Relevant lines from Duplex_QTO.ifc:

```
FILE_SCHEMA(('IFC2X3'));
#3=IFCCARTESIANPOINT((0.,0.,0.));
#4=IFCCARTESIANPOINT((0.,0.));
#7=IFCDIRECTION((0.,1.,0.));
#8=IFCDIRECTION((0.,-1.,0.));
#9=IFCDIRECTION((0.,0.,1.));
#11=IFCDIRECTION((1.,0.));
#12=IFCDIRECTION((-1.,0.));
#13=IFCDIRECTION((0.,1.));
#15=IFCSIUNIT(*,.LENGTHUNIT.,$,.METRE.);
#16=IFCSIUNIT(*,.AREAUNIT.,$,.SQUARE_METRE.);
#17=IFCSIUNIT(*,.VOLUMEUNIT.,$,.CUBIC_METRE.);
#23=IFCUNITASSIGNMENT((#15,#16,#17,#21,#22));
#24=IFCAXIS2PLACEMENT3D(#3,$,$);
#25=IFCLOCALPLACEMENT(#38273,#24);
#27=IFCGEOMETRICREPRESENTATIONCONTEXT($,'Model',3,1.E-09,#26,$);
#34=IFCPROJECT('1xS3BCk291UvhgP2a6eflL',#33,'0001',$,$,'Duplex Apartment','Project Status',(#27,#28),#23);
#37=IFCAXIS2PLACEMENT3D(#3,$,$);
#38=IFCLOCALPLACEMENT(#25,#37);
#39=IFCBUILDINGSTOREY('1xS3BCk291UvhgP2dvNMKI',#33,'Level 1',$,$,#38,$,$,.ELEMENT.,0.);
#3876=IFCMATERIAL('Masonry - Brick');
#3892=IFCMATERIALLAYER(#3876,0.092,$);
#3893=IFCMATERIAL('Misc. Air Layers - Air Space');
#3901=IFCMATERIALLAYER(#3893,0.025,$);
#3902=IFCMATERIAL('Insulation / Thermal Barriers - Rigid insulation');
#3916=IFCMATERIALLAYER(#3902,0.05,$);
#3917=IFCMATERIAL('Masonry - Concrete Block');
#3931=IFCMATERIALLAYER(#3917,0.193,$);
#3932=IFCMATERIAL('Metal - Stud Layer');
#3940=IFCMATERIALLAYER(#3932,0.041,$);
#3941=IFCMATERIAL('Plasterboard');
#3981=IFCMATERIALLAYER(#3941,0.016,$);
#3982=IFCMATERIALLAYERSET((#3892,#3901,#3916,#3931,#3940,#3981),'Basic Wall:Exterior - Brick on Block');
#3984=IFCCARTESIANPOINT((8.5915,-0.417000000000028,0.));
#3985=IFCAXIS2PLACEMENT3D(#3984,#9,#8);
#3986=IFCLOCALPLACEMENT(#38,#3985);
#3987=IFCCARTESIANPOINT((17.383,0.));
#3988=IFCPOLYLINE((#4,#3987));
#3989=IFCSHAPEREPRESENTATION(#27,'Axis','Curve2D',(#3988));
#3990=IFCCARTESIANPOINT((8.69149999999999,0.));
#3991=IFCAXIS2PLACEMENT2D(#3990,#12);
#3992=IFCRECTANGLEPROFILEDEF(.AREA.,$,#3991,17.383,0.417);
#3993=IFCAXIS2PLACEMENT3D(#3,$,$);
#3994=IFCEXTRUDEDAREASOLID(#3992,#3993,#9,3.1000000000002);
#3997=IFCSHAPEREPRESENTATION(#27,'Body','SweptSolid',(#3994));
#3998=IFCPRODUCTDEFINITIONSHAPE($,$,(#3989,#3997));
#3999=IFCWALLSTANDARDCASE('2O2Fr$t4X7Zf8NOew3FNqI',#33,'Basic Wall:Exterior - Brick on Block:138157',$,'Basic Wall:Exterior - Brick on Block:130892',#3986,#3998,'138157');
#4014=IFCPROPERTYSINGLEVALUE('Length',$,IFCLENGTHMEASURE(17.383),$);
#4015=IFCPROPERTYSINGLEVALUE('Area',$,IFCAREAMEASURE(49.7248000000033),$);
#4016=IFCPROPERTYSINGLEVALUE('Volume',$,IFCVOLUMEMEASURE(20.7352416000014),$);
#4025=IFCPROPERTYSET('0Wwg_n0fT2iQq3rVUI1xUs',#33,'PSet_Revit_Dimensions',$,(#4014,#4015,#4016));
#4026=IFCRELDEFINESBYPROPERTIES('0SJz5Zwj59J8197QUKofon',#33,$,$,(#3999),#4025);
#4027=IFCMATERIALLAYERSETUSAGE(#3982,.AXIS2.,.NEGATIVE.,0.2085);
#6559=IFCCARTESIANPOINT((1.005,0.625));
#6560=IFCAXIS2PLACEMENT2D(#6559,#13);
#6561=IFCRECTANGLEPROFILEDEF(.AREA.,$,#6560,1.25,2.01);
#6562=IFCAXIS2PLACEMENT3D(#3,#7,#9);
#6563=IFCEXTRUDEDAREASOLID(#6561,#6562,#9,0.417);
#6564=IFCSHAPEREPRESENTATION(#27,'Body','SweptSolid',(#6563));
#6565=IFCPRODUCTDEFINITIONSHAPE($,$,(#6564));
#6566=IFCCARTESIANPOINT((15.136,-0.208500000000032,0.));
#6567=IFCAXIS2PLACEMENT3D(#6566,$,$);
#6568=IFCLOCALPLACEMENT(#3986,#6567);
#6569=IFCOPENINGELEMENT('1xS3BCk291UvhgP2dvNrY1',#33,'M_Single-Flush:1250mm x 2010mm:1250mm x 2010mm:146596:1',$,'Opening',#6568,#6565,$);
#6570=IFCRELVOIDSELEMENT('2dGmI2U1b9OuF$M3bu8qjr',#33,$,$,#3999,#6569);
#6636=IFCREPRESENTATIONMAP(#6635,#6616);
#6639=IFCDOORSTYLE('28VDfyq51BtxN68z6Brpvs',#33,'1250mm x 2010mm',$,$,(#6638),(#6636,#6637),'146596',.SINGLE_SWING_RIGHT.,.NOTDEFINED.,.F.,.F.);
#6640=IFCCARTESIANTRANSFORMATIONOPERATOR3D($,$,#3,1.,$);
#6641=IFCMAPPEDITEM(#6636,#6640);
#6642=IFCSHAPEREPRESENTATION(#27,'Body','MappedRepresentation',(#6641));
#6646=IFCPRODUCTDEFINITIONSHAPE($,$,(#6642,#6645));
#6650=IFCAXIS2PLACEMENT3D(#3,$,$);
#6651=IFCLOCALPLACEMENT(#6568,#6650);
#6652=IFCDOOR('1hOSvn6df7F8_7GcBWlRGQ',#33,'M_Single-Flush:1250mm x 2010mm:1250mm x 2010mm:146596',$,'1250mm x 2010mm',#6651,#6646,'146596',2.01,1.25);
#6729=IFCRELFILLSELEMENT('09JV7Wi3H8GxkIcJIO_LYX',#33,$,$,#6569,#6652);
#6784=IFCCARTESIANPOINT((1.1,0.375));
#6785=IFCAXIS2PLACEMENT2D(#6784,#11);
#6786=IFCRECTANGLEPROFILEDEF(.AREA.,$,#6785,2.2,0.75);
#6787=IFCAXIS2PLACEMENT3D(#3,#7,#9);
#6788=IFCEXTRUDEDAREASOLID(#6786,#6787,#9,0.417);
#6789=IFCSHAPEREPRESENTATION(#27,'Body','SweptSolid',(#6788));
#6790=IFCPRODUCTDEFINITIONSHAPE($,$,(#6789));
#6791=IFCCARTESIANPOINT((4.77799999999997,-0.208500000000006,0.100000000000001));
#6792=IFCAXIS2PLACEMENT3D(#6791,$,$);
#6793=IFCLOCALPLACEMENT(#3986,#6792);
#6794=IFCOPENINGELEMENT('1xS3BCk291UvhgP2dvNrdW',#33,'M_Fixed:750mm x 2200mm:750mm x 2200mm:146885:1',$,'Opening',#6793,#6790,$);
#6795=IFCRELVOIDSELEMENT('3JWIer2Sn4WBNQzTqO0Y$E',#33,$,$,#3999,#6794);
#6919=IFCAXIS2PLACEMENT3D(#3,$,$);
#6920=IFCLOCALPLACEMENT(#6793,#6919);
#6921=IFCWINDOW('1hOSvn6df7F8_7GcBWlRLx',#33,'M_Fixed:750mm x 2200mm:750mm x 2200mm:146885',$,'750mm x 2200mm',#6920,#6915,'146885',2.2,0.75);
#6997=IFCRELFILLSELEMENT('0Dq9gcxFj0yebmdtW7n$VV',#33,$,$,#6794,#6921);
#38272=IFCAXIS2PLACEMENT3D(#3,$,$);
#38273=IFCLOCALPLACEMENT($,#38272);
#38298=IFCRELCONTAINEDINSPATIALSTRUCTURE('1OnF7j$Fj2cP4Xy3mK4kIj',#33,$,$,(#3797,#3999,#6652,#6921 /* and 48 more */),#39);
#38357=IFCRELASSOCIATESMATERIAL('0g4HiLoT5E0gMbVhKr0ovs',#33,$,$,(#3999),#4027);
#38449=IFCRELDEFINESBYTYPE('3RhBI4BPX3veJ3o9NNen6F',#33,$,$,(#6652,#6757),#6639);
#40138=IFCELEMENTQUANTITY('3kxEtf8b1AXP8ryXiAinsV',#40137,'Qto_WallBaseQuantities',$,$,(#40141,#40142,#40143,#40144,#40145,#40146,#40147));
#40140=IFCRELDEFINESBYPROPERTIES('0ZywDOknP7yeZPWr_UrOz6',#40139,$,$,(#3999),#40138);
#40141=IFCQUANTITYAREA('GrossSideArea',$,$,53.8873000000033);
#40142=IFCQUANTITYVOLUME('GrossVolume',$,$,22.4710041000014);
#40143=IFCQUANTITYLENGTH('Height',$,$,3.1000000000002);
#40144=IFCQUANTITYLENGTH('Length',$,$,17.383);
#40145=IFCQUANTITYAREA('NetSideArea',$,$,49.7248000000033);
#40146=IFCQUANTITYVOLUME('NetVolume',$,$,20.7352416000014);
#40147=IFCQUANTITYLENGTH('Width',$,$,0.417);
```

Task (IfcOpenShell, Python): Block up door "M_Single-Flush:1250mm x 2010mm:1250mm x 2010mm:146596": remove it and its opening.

```python
import ifcopenshell
import ifcopenshell.api.feature
import ifcopenshell.api.pset
import ifcopenshell.api.root
import ifcopenshell.geom
import ifcopenshell.util.element
import ifcopenshell.util.shape
import ifcopenshell.util.unit

model = ifcopenshell.open("Duplex_QTO.ifc")
area_scale = ifcopenshell.util.unit.calculate_unit_scale(model, "AREAUNIT")
volume_scale = ifcopenshell.util.unit.calculate_unit_scale(model, "VOLUMEUNIT")
settings = ifcopenshell.geom.settings()


def volume(element):
    """Net volume in cubic metres, openings subtracted."""
    shape = ifcopenshell.geom.create_shape(settings, element)
    return ifcopenshell.util.shape.get_volume(shape.geometry)


door = model.by_guid("1hOSvn6df7F8_7GcBWlRGQ")
opening = door.FillsVoids[0].RelatingOpeningElement
wall = opening.VoidsElements[0].RelatingBuildingElement
before = volume(wall)

ifcopenshell.api.root.remove_product(model, product=door)
ifcopenshell.api.feature.remove_feature(model, feature=opening)

after = volume(wall)
thickness = 0.417  # wall thickness in metres

# Update the wall's stored quantities.
pset = model.by_id(ifcopenshell.util.element.get_pset(wall, "PSet_Revit_Dimensions", should_inherit=False)["id"])
ifcopenshell.api.pset.edit_pset(model, pset=pset, properties={
    "Area": model.create_entity("IfcAreaMeasure", after / thickness / area_scale),
    "Volume": model.create_entity("IfcVolumeMeasure", after / volume_scale),
})
qto = model.by_id(ifcopenshell.util.element.get_pset(wall, "Qto_WallBaseQuantities", should_inherit=False)["id"])
ifcopenshell.api.pset.edit_qto(model, qto=qto, properties={
    "NetSideArea": after / thickness / area_scale,
    "NetVolume": after / volume_scale,
})

print(f"wall volume {before:.3f} -> {after:.3f} m3")

model.write("Duplex_QTO_v2.ifc")
```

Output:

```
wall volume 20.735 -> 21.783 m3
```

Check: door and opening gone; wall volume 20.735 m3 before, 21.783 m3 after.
